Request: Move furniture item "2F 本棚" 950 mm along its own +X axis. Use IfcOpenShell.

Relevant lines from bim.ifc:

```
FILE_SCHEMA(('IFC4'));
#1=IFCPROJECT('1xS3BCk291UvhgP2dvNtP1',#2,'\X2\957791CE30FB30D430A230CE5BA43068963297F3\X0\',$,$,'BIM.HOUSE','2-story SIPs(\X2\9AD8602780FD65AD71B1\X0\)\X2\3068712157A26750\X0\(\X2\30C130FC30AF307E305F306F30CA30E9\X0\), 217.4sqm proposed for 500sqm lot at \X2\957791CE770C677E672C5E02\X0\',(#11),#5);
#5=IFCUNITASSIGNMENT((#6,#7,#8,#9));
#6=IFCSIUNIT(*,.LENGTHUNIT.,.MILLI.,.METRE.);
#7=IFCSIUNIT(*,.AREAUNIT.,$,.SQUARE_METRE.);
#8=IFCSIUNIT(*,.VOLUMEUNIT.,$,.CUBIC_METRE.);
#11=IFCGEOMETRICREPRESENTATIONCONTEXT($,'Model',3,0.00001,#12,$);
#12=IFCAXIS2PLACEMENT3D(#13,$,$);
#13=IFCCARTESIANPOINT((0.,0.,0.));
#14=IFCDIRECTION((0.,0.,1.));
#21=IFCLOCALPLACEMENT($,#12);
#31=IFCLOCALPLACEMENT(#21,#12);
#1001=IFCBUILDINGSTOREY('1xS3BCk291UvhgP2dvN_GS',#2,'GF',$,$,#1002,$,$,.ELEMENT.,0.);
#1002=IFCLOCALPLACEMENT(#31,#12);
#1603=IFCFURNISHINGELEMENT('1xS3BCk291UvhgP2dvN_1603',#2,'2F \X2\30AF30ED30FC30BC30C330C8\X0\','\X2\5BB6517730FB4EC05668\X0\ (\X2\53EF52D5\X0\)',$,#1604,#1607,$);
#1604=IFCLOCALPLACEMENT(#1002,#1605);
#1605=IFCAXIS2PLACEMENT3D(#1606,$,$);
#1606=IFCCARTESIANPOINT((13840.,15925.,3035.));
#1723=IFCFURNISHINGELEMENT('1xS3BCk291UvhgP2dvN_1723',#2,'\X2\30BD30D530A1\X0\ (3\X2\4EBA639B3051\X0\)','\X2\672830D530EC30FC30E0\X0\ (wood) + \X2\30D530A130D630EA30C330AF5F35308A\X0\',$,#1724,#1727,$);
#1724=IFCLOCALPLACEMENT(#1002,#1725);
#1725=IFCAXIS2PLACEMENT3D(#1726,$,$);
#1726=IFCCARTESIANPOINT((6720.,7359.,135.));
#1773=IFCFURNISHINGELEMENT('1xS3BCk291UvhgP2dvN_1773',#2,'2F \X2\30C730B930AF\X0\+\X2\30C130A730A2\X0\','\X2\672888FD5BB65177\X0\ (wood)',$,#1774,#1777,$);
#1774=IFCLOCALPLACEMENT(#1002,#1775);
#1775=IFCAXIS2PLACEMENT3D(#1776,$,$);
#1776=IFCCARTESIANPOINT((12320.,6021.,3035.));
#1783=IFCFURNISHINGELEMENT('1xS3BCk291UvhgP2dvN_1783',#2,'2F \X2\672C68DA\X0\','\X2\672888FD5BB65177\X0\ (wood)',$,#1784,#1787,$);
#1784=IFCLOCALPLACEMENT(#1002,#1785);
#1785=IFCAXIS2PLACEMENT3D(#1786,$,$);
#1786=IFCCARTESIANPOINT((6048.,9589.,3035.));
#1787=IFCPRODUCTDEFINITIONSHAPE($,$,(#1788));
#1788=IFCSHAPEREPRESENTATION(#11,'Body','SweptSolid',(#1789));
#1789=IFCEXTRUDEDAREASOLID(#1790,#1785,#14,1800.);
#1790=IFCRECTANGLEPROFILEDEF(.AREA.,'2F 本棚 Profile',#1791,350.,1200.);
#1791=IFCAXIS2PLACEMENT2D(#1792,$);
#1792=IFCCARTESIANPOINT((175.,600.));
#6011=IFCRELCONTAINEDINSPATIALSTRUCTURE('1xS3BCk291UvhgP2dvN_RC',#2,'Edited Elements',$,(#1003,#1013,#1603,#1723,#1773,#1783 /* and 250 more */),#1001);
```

```python
import ifcopenshell
import ifcopenshell.api.geometry
import ifcopenshell.util.placement
import ifcopenshell.util.unit

model = ifcopenshell.open("bim.ifc")
unit_scale = ifcopenshell.util.unit.calculate_unit_scale(model)

item = model.by_guid("1xS3BCk291UvhgP2dvN_1783")
matrix = ifcopenshell.util.placement.get_local_placement(item.ObjectPlacement)
matrix[:3, 3] += matrix[:3, 0] * 0.95 / unit_scale
ifcopenshell.api.geometry.edit_object_placement(model, product=item, matrix=matrix, is_si=False)

print(ifcopenshell.util.placement.get_local_placement(item.ObjectPlacement).round(3) + 0.0)

model.write("bim_v2.ifc")
```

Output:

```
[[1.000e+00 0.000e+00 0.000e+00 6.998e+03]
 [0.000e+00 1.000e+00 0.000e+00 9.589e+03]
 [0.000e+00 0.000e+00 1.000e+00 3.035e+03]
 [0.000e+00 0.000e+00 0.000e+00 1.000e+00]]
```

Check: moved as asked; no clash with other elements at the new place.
